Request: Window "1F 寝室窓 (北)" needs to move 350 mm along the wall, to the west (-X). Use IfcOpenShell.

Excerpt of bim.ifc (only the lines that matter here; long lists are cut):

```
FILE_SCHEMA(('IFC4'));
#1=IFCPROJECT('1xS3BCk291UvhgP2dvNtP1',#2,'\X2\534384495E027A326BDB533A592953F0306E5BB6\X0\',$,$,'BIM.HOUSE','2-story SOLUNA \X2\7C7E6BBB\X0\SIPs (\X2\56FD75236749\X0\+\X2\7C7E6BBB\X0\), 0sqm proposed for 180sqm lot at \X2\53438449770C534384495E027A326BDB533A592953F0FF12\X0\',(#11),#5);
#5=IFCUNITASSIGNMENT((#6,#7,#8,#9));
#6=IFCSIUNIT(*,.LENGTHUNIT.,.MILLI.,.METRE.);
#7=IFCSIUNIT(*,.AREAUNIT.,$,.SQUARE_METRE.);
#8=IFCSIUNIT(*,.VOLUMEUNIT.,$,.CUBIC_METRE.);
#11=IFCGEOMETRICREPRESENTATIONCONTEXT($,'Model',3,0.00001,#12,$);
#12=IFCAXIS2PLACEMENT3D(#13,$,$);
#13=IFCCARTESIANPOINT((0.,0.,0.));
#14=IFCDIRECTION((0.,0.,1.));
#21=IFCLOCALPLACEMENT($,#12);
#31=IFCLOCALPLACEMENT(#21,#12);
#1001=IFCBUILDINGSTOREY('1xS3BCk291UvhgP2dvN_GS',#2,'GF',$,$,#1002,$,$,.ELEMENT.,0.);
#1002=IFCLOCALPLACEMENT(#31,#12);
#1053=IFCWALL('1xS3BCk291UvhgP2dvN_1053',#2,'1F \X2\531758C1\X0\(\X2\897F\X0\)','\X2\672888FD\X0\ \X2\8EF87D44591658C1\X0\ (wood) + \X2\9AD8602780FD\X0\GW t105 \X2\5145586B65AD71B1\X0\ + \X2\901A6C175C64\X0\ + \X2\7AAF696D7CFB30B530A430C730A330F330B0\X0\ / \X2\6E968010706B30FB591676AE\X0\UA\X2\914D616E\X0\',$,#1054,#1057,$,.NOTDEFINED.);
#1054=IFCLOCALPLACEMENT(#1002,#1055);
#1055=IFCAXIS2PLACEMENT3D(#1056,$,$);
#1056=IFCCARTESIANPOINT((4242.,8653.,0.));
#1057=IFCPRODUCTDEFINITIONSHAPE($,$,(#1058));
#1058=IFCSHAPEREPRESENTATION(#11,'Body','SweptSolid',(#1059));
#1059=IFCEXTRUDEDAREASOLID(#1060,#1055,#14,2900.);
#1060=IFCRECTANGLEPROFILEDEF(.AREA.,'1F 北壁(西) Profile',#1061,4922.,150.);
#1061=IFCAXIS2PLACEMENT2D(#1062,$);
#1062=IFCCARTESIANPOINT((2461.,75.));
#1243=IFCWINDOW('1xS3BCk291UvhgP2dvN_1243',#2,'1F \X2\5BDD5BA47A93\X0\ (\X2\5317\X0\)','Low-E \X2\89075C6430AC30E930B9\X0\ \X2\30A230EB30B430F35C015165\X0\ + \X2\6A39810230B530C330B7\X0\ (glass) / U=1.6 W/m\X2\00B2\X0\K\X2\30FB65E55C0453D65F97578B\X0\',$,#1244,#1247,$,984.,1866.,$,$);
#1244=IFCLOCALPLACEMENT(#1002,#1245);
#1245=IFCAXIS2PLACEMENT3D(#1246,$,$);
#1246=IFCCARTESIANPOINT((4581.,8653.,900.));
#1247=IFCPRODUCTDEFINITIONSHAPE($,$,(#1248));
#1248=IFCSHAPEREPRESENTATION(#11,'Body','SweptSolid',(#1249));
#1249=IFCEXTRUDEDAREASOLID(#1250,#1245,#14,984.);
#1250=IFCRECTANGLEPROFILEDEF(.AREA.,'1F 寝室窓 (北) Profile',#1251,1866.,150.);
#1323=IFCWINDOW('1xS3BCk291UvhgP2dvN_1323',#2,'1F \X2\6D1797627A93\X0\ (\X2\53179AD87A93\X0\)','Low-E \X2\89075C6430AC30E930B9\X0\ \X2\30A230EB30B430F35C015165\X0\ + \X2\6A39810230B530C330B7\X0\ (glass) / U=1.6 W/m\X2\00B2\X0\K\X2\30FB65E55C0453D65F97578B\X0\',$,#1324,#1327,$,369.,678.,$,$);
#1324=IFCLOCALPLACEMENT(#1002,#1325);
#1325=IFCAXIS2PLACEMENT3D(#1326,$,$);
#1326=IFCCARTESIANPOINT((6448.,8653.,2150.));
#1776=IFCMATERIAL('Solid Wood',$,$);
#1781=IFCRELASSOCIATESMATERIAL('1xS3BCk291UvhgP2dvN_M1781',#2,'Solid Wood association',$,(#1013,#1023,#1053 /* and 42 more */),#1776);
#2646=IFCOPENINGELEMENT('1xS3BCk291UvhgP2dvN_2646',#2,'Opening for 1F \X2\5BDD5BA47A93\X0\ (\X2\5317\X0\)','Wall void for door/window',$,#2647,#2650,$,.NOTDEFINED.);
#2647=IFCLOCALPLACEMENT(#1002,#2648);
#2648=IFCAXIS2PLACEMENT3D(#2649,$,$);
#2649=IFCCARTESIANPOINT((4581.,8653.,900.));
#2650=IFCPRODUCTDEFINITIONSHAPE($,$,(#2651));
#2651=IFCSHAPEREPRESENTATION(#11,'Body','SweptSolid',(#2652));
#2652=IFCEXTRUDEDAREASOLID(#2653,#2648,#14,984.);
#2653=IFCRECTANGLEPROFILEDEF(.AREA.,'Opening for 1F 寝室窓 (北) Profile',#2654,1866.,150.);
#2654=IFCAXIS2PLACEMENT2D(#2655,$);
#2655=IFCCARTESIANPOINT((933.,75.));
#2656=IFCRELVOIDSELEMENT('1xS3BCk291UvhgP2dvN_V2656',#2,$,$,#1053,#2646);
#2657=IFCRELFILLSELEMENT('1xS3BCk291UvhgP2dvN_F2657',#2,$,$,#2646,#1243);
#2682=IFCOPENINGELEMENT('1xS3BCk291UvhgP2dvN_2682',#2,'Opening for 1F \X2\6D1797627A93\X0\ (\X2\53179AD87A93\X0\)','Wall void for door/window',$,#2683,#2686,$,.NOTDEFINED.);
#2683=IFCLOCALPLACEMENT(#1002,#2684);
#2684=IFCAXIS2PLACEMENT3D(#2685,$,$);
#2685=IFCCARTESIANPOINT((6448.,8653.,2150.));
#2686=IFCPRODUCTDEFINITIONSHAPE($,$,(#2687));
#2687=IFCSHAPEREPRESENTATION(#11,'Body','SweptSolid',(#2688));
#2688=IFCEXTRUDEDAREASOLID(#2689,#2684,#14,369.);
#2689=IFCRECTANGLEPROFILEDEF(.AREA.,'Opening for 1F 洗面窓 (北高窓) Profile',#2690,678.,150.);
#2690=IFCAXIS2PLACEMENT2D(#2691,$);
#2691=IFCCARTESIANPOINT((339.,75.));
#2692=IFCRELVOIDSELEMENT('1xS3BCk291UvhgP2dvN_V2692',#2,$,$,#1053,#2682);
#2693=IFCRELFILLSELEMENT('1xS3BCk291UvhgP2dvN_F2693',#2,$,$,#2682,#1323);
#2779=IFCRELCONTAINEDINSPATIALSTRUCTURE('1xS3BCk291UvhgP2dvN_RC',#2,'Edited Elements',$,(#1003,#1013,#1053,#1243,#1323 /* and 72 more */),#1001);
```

```python
import ifcopenshell
import ifcopenshell.api.geometry
import ifcopenshell.util.placement
import ifcopenshell.util.unit

model = ifcopenshell.open("bim.ifc")
unit_scale = ifcopenshell.util.unit.calculate_unit_scale(model)

window = model.by_id(1243)
opening = window.FillsVoids[0].RelatingOpeningElement
wall = opening.VoidsElements[0].RelatingBuildingElement

wall_matrix = ifcopenshell.util.placement.get_local_placement(wall.ObjectPlacement)
shift = wall_matrix[:3, 0] * -0.35 / unit_scale
before = ifcopenshell.util.placement.get_local_placement(window.ObjectPlacement)[:3, 3].copy()

# The window is not placed relative to its opening, so move both.
for product in (opening, window):
    matrix = ifcopenshell.util.placement.get_local_placement(product.ObjectPlacement)
    matrix[:3, 3] += shift
    ifcopenshell.api.geometry.edit_object_placement(model, product=product, matrix=matrix, is_si=False)

after = ifcopenshell.util.placement.get_local_placement(window.ObjectPlacement)[:3, 3]
print("window moved by", (after - before).round(3) + 0.0)

model.write("bim_v2.ifc")
```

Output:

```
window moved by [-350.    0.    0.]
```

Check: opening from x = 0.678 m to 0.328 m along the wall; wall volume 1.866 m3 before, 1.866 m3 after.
